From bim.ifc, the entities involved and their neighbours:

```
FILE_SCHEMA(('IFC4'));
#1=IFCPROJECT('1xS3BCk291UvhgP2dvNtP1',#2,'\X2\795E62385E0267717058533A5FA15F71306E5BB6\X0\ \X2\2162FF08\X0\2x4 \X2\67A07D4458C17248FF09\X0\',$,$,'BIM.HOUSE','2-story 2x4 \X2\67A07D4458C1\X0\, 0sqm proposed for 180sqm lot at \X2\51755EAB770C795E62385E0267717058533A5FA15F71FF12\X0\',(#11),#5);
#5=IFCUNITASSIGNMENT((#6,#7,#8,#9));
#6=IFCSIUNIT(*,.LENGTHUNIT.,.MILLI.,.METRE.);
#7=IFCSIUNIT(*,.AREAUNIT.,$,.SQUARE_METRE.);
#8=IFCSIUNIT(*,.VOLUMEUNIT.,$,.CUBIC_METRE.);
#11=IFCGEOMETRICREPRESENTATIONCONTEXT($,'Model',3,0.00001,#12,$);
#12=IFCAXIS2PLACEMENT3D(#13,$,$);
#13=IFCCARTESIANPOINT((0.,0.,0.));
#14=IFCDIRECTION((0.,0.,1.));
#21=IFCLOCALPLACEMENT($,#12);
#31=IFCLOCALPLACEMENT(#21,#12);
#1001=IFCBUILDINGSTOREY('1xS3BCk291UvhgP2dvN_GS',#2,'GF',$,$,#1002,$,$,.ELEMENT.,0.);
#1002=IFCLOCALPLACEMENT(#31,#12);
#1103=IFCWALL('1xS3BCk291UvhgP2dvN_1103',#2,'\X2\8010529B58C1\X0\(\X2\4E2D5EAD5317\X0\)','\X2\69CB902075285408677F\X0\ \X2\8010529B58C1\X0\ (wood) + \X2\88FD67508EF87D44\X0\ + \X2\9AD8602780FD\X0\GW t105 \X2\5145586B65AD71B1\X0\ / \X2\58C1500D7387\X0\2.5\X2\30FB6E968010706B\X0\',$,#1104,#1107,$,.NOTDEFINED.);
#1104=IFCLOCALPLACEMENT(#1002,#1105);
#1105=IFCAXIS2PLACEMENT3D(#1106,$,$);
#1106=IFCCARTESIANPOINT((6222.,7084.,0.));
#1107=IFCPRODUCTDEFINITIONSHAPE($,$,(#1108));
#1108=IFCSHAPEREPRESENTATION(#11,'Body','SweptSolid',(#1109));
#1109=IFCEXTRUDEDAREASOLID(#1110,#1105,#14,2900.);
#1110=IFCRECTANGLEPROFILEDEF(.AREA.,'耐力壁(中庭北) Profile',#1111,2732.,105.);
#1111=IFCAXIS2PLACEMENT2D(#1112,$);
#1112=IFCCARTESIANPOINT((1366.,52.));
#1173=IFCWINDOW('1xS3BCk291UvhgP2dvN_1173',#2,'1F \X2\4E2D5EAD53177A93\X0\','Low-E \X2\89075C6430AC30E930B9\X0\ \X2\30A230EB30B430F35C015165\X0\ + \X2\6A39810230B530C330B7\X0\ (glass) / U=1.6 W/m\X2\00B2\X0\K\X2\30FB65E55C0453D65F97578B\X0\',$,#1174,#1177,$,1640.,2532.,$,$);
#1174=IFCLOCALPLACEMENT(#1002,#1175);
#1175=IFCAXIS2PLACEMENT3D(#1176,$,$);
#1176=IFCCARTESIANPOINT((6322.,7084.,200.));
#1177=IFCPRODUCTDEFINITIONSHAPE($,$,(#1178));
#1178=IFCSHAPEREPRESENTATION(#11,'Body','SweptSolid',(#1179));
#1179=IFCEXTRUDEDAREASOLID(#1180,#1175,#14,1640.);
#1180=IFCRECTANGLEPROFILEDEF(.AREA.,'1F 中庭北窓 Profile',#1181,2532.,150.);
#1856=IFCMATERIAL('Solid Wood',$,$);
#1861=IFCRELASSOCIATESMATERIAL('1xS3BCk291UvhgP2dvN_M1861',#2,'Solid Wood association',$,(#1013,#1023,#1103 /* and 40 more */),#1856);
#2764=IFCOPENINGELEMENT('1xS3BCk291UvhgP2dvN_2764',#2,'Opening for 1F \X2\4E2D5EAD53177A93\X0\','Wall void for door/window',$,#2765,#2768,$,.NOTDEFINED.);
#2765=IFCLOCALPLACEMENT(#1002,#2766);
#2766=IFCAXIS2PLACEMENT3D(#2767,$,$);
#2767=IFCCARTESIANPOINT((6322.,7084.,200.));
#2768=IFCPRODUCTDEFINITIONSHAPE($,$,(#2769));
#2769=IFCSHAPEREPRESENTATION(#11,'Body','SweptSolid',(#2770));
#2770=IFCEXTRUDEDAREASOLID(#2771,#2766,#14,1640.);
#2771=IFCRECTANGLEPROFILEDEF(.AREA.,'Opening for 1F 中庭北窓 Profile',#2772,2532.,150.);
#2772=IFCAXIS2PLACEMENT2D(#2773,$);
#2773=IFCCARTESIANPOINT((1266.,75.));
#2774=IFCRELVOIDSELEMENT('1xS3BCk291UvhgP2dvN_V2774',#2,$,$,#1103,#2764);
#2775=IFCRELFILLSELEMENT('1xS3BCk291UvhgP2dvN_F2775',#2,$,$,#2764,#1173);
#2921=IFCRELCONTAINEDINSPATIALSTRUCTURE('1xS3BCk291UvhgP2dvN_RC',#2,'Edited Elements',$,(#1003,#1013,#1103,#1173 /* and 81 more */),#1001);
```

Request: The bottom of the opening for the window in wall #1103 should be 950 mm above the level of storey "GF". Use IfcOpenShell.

```python
import numpy as np
import ifcopenshell
import ifcopenshell.api.geometry
import ifcopenshell.geom
import ifcopenshell.util.element
import ifcopenshell.util.placement
import ifcopenshell.util.shape
import ifcopenshell.util.unit

model = ifcopenshell.open("bim.ifc")
unit_scale = ifcopenshell.util.unit.calculate_unit_scale(model)

window = model.by_guid("1xS3BCk291UvhgP2dvN_1173")
opening = window.FillsVoids[0].RelatingOpeningElement
storey = ifcopenshell.util.element.get_container(window, ifc_class="IfcBuildingStorey")
level = ifcopenshell.util.placement.get_local_placement(storey.ObjectPlacement)[2, 3]

# The opening's origin need not be at the sill, so measure its lowest point.
shape = ifcopenshell.geom.create_shape(ifcopenshell.geom.settings(), opening)
bottom = ifcopenshell.util.shape.get_shape_bottom_elevation(shape, shape.geometry) / unit_scale
dz = level + 0.95 / unit_scale - bottom

shift = np.array([0.0, 0.0, dz])
# The window is not placed relative to its opening, so move both.
for product in (opening, window):
    matrix = ifcopenshell.util.placement.get_local_placement(product.ObjectPlacement)
    matrix[:3, 3] += shift
    ifcopenshell.api.geometry.edit_object_placement(model, product=product, matrix=matrix, is_si=False)

print(f"moved by {dz * unit_scale:+.3f} m")

model.write("bim_edited.ifc")
```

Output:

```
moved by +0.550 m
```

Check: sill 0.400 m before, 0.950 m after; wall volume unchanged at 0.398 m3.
